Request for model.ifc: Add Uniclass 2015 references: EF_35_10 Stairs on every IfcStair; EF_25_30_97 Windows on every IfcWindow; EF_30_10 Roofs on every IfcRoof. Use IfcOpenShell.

First a look at what the model holds.

```python
import ifcopenshell

model = ifcopenshell.open("model.ifc")
print(model.schema)
print("classifications:", [c.Name for c in model.by_type("IfcClassification")])
for ifc_class in ("IfcDoor", "IfcRoof", "IfcStair", "IfcWall", "IfcWindow"):
    print(ifc_class, len(model.by_type(ifc_class)))
```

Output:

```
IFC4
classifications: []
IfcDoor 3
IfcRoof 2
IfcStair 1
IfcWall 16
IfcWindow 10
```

```python
import ifcopenshell
import ifcopenshell.api.classification

model = ifcopenshell.open("model.ifc")

system = ifcopenshell.api.classification.add_classification(model, classification="Uniclass 2015")

codes = {
    "IfcStair": ("EF_35_10", "Stairs"),
    "IfcWindow": ("EF_25_30_97", "Windows"),
    "IfcRoof": ("EF_30_10", "Roofs"),
}
for ifc_class, (code, name) in codes.items():
    products = model.by_type(ifc_class)
    ifcopenshell.api.classification.add_reference(
        model, products=products, classification=system, identification=code, name=name
    )
    print(code, len(products))

model.write("model_updated.ifc")
```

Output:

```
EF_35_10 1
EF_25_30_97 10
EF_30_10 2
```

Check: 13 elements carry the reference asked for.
